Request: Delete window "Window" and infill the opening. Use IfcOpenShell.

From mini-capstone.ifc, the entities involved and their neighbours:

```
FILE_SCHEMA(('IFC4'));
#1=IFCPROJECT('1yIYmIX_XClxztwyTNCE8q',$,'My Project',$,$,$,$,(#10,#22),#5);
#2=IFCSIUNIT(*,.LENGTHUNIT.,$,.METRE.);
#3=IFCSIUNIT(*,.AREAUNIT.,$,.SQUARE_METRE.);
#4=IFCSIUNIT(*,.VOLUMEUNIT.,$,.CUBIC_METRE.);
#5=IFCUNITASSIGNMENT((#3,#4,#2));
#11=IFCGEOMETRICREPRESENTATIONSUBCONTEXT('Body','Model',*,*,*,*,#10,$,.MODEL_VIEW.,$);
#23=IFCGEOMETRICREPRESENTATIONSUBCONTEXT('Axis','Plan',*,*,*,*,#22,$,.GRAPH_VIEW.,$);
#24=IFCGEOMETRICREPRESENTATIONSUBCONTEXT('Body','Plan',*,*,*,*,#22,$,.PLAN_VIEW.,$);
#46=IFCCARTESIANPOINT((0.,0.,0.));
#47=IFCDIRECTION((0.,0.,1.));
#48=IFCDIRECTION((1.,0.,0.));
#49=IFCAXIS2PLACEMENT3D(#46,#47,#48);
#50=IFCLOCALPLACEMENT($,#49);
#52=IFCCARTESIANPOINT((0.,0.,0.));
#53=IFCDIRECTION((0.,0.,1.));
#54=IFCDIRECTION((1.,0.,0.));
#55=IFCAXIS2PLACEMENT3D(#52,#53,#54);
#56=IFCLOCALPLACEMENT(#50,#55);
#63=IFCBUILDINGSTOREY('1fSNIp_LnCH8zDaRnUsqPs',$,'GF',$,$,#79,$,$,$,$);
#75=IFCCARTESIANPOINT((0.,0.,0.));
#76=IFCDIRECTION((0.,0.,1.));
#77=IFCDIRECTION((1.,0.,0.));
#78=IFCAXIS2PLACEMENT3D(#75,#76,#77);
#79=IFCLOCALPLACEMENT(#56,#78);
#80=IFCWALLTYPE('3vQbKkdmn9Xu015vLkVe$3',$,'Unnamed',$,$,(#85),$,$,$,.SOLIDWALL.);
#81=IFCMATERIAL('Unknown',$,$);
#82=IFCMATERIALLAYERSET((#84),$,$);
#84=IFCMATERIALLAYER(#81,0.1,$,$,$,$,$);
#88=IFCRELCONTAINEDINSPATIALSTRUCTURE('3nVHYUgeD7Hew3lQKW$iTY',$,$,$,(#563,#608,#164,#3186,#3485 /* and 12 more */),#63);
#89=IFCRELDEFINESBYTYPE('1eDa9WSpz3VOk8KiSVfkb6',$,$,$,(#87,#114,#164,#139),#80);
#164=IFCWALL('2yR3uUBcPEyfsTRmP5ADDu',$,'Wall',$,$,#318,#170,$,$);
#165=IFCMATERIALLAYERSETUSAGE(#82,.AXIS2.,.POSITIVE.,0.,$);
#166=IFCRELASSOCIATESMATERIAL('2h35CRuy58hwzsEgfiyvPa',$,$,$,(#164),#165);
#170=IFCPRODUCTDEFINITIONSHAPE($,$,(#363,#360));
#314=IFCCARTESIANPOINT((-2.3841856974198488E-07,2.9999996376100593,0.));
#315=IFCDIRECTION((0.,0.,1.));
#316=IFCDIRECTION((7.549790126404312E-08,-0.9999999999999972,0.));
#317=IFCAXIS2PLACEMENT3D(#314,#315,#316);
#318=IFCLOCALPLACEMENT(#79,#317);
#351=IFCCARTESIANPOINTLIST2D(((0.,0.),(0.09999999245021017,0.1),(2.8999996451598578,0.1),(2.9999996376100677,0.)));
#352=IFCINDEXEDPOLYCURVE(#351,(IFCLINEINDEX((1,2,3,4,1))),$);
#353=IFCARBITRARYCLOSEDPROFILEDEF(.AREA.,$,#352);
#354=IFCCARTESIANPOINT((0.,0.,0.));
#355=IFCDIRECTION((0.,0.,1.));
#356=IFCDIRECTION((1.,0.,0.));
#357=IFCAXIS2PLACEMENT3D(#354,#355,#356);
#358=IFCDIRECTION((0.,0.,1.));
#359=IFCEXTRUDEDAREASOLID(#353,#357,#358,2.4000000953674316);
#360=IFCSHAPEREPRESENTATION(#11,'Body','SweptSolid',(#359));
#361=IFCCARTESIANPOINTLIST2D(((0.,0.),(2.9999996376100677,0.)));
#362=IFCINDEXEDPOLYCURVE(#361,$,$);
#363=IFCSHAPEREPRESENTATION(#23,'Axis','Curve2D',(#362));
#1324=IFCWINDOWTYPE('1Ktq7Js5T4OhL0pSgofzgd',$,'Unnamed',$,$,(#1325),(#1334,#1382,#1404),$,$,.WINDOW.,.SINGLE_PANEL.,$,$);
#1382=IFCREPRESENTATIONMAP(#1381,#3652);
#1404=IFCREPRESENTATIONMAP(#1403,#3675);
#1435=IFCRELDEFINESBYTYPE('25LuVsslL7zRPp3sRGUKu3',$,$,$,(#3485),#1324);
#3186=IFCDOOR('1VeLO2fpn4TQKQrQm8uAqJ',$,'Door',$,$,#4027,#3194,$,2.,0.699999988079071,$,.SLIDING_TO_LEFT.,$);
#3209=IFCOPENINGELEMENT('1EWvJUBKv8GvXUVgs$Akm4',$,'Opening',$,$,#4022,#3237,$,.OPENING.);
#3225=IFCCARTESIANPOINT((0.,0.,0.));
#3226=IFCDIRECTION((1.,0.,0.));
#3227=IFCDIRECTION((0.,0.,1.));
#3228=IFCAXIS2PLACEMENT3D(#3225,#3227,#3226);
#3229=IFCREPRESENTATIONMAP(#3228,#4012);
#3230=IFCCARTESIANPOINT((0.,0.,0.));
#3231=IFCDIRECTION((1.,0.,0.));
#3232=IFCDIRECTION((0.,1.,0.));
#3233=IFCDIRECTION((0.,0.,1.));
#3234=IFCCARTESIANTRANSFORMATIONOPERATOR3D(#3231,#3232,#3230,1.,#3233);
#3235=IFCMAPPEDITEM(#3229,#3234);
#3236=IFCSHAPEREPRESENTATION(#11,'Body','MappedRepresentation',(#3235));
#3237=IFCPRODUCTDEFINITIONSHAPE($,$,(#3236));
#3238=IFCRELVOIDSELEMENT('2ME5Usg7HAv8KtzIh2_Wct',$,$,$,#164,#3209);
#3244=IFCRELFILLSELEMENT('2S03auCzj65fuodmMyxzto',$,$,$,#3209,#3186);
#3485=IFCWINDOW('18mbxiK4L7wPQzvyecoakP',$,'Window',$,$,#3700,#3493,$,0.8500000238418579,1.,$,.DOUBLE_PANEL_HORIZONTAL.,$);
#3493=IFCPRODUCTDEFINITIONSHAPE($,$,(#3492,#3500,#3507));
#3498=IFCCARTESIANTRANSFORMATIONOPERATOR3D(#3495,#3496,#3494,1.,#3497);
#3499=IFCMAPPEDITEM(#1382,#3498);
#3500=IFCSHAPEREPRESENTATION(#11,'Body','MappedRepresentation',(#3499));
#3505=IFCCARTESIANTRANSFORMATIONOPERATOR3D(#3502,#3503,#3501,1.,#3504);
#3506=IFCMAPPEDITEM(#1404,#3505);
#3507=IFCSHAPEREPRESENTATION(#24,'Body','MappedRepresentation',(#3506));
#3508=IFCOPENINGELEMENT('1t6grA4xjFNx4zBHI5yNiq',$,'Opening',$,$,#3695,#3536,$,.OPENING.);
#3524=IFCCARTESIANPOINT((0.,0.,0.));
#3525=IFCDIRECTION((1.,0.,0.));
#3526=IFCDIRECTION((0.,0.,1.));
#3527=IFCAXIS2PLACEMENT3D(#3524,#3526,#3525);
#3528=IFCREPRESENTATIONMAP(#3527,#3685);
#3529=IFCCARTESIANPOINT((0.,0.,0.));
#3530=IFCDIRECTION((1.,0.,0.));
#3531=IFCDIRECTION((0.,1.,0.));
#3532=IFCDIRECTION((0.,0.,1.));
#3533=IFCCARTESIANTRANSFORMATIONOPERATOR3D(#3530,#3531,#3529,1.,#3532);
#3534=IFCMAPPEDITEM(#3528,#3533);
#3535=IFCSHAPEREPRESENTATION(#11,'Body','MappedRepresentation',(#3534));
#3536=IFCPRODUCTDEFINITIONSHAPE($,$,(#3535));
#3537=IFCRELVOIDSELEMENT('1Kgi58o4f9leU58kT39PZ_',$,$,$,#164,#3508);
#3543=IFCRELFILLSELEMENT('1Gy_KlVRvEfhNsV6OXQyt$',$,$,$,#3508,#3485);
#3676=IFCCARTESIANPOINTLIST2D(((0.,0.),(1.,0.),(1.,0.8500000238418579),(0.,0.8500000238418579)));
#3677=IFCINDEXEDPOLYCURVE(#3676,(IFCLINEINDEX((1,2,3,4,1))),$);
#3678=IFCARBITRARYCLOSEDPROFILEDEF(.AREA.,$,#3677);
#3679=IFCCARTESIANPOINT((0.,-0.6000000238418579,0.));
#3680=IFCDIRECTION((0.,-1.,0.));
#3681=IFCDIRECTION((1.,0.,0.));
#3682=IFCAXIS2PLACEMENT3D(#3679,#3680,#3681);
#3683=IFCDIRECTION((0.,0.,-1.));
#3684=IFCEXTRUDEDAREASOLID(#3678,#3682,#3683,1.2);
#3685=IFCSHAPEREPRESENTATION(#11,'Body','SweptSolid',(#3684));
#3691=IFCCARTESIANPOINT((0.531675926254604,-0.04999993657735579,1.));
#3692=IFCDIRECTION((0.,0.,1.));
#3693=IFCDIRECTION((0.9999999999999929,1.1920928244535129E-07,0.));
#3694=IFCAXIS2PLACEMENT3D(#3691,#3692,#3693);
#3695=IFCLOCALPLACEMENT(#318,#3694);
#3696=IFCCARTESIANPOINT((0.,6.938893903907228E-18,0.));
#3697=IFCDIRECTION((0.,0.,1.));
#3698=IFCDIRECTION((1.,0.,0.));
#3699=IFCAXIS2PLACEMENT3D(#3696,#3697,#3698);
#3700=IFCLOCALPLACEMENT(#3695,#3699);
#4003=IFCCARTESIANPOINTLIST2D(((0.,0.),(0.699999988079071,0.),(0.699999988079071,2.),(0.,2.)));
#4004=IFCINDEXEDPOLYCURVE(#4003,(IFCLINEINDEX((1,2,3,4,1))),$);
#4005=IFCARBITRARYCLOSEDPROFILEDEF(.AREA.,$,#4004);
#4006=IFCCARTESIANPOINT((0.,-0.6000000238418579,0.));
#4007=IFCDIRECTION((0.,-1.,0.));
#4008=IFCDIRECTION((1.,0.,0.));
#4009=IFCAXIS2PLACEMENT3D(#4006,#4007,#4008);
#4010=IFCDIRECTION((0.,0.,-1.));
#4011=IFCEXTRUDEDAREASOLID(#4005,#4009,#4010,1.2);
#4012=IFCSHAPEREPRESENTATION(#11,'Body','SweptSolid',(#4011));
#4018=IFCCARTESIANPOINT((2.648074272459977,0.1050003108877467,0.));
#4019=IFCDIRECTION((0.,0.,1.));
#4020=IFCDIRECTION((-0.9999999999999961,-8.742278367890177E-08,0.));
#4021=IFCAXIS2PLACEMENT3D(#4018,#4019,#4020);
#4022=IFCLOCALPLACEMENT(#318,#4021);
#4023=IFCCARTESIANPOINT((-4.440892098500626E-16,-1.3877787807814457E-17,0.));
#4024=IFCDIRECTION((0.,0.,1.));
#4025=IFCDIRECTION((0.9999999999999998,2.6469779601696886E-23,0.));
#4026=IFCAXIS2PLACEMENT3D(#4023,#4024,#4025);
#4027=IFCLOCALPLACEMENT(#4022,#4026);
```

```python
import ifcopenshell
import ifcopenshell.api.feature
import ifcopenshell.api.root
import ifcopenshell.geom
import ifcopenshell.util.shape

model = ifcopenshell.open("mini-capstone.ifc")
settings = ifcopenshell.geom.settings()


def volume(element):
    """Net volume in cubic metres, openings subtracted."""
    shape = ifcopenshell.geom.create_shape(settings, element)
    return ifcopenshell.util.shape.get_volume(shape.geometry)


window = model.by_guid("18mbxiK4L7wPQzvyecoakP")
opening = window.FillsVoids[0].RelatingOpeningElement
wall = opening.VoidsElements[0].RelatingBuildingElement
before = volume(wall)

ifcopenshell.api.root.remove_product(model, product=window)
ifcopenshell.api.feature.remove_feature(model, feature=opening)

after = volume(wall)

print(f"wall volume {before:.3f} -> {after:.3f} m3")

model.write("mini-capstone-out.ifc")
```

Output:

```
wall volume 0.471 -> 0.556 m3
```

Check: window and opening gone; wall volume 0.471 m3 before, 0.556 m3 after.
